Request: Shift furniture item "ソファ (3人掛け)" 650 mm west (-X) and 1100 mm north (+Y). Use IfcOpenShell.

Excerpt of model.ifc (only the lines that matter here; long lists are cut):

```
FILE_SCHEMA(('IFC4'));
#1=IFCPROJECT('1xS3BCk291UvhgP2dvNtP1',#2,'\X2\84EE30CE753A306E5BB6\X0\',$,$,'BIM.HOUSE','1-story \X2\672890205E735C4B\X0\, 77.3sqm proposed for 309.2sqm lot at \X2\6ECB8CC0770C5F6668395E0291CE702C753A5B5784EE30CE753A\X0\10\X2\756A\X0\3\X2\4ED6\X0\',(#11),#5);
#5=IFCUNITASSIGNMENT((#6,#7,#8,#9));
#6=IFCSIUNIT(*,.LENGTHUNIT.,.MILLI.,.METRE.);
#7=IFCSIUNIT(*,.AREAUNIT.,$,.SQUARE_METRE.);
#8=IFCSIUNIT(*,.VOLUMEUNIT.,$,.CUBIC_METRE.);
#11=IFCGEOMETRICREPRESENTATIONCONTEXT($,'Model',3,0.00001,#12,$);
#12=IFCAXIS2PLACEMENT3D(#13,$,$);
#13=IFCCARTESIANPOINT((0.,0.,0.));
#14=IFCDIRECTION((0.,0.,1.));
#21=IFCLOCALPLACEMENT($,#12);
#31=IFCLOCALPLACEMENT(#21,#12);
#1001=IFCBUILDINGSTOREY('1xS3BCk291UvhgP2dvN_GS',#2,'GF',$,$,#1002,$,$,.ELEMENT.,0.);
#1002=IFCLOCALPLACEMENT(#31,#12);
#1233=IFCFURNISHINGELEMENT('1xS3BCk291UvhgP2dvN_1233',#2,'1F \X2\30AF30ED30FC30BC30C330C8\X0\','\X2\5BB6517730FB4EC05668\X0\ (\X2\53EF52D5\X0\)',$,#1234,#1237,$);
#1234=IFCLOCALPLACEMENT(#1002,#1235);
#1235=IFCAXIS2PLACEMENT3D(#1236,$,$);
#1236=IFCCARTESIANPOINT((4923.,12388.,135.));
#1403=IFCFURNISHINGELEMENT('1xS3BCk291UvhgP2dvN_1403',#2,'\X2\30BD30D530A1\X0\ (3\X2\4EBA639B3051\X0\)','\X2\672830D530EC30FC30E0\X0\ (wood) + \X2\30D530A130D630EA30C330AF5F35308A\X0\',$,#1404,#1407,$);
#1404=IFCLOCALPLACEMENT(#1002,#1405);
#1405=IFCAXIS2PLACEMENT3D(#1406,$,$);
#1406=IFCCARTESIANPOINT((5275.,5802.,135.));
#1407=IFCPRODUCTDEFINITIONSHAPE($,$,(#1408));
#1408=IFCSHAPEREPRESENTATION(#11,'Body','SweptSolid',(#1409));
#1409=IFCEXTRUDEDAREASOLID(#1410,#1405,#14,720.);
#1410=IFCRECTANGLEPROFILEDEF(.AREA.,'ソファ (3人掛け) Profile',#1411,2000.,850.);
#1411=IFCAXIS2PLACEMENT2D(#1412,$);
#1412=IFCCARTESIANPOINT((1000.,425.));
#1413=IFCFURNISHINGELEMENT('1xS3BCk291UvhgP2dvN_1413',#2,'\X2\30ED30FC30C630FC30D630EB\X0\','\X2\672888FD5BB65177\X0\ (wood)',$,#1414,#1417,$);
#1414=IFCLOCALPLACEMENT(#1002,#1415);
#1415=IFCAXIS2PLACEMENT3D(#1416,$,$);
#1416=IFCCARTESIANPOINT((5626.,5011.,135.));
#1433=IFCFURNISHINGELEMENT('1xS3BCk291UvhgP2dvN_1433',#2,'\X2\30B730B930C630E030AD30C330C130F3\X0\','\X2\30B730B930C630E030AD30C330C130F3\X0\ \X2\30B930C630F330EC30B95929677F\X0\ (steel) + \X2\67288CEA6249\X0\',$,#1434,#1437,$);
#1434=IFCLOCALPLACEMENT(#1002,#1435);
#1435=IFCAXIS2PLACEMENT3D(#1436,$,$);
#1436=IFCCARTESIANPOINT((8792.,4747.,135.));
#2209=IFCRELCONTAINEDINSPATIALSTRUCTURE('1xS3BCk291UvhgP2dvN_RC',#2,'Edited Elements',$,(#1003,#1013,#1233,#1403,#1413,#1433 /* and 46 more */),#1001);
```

```python
import ifcopenshell
import ifcopenshell.api.geometry
import ifcopenshell.util.placement

model = ifcopenshell.open("model.ifc")

item = model.by_id(1403)
matrix = ifcopenshell.util.placement.get_local_placement(item.ObjectPlacement)
matrix[0, 3] -= 650.0
matrix[1, 3] += 1100.0
ifcopenshell.api.geometry.edit_object_placement(model, product=item, matrix=matrix, is_si=False)

print(ifcopenshell.util.placement.get_local_placement(item.ObjectPlacement).round(3) + 0.0)

model.write("model_edited.ifc")
```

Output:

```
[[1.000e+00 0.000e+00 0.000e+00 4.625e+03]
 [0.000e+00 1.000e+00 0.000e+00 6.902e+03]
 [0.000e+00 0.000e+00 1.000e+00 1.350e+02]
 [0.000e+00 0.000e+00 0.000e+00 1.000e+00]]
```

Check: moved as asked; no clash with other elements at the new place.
